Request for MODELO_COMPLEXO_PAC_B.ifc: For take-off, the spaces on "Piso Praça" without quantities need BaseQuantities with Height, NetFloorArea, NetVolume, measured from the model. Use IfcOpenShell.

First a look at what the model holds.

```python
import ifcopenshell
import ifcopenshell.util.element
import ifcopenshell.util.unit

model = ifcopenshell.open("MODELO_COMPLEXO_PAC_B.ifc")
print(model.schema)
for unit_type in ("LENGTHUNIT", "AREAUNIT", "VOLUMEUNIT"):
    print(unit_type, ifcopenshell.util.unit.calculate_unit_scale(model, unit_type))
storey = next(s for s in model.by_type("IfcBuildingStorey") if s.Name == "Piso Praça")
spaces = [e for e in ifcopenshell.util.element.get_decomposition(storey) if e.is_a("IfcSpace")]
for e in sorted(spaces, key=lambda e: e.id()):
    print(e.id(), e.is_a(), e.Name, list(ifcopenshell.util.element.get_psets(e, qtos_only=True)), sep=" | ")
```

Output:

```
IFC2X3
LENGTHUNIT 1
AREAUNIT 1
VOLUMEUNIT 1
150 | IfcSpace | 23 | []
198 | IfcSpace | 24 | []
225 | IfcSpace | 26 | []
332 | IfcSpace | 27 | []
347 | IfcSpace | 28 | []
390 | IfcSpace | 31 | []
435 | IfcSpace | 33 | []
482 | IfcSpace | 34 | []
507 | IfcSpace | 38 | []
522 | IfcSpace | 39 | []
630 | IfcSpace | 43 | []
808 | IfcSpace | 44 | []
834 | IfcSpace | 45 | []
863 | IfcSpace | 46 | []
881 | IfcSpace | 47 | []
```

```python
import ifcopenshell
import ifcopenshell.api.pset
import ifcopenshell.geom
import ifcopenshell.util.element
import ifcopenshell.util.shape
import ifcopenshell.util.unit

model = ifcopenshell.open("MODELO_COMPLEXO_PAC_B.ifc")
unit_scale = ifcopenshell.util.unit.calculate_unit_scale(model)
area_scale = ifcopenshell.util.unit.calculate_unit_scale(model, "AREAUNIT")
volume_scale = ifcopenshell.util.unit.calculate_unit_scale(model, "VOLUMEUNIT")
settings = ifcopenshell.geom.settings()

storey = next(s for s in model.by_type("IfcBuildingStorey") if s.Name == "Piso Praça")
spaces = [e for e in ifcopenshell.util.element.get_decomposition(storey) if e.is_a("IfcSpace")]

for e in sorted(spaces, key=lambda e: e.id()):
    if ifcopenshell.util.element.get_psets(e, qtos_only=True, should_inherit=False):
        continue
    # Geometry comes back in metres, in the element's own axes.
    shape = ifcopenshell.geom.create_shape(settings, e)
    values = {
        "Height": ifcopenshell.util.shape.get_z(shape.geometry) / unit_scale,
        "NetFloorArea": ifcopenshell.util.shape.get_footprint_area(shape.geometry) / area_scale,
        "NetVolume": ifcopenshell.util.shape.get_volume(shape.geometry) / volume_scale,
    }
    qto = ifcopenshell.api.pset.add_qto(model, product=e, name="BaseQuantities")
    ifcopenshell.api.pset.edit_qto(model, qto=qto, properties=values)
    print(e.id(), {k: round(v, 3) for k, v in values.items()})

model.write("MODELO_COMPLEXO_PAC_B_edited.ifc")
```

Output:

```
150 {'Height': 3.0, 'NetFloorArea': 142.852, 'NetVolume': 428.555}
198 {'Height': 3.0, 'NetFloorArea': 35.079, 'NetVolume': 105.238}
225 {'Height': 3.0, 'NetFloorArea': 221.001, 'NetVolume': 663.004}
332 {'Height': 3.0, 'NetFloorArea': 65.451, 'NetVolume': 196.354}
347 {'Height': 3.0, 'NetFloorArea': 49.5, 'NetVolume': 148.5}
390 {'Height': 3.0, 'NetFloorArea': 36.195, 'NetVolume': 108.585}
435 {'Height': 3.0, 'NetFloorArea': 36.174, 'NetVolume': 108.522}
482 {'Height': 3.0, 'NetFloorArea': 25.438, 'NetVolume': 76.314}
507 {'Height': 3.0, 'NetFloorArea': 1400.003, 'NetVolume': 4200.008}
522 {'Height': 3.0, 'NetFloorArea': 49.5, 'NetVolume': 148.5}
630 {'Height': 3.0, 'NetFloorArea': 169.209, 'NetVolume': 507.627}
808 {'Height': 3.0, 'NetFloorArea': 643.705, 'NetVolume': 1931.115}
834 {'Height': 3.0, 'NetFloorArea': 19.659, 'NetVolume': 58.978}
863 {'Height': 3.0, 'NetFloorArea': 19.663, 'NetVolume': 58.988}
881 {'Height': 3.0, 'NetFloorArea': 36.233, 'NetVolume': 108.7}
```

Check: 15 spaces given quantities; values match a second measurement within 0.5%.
